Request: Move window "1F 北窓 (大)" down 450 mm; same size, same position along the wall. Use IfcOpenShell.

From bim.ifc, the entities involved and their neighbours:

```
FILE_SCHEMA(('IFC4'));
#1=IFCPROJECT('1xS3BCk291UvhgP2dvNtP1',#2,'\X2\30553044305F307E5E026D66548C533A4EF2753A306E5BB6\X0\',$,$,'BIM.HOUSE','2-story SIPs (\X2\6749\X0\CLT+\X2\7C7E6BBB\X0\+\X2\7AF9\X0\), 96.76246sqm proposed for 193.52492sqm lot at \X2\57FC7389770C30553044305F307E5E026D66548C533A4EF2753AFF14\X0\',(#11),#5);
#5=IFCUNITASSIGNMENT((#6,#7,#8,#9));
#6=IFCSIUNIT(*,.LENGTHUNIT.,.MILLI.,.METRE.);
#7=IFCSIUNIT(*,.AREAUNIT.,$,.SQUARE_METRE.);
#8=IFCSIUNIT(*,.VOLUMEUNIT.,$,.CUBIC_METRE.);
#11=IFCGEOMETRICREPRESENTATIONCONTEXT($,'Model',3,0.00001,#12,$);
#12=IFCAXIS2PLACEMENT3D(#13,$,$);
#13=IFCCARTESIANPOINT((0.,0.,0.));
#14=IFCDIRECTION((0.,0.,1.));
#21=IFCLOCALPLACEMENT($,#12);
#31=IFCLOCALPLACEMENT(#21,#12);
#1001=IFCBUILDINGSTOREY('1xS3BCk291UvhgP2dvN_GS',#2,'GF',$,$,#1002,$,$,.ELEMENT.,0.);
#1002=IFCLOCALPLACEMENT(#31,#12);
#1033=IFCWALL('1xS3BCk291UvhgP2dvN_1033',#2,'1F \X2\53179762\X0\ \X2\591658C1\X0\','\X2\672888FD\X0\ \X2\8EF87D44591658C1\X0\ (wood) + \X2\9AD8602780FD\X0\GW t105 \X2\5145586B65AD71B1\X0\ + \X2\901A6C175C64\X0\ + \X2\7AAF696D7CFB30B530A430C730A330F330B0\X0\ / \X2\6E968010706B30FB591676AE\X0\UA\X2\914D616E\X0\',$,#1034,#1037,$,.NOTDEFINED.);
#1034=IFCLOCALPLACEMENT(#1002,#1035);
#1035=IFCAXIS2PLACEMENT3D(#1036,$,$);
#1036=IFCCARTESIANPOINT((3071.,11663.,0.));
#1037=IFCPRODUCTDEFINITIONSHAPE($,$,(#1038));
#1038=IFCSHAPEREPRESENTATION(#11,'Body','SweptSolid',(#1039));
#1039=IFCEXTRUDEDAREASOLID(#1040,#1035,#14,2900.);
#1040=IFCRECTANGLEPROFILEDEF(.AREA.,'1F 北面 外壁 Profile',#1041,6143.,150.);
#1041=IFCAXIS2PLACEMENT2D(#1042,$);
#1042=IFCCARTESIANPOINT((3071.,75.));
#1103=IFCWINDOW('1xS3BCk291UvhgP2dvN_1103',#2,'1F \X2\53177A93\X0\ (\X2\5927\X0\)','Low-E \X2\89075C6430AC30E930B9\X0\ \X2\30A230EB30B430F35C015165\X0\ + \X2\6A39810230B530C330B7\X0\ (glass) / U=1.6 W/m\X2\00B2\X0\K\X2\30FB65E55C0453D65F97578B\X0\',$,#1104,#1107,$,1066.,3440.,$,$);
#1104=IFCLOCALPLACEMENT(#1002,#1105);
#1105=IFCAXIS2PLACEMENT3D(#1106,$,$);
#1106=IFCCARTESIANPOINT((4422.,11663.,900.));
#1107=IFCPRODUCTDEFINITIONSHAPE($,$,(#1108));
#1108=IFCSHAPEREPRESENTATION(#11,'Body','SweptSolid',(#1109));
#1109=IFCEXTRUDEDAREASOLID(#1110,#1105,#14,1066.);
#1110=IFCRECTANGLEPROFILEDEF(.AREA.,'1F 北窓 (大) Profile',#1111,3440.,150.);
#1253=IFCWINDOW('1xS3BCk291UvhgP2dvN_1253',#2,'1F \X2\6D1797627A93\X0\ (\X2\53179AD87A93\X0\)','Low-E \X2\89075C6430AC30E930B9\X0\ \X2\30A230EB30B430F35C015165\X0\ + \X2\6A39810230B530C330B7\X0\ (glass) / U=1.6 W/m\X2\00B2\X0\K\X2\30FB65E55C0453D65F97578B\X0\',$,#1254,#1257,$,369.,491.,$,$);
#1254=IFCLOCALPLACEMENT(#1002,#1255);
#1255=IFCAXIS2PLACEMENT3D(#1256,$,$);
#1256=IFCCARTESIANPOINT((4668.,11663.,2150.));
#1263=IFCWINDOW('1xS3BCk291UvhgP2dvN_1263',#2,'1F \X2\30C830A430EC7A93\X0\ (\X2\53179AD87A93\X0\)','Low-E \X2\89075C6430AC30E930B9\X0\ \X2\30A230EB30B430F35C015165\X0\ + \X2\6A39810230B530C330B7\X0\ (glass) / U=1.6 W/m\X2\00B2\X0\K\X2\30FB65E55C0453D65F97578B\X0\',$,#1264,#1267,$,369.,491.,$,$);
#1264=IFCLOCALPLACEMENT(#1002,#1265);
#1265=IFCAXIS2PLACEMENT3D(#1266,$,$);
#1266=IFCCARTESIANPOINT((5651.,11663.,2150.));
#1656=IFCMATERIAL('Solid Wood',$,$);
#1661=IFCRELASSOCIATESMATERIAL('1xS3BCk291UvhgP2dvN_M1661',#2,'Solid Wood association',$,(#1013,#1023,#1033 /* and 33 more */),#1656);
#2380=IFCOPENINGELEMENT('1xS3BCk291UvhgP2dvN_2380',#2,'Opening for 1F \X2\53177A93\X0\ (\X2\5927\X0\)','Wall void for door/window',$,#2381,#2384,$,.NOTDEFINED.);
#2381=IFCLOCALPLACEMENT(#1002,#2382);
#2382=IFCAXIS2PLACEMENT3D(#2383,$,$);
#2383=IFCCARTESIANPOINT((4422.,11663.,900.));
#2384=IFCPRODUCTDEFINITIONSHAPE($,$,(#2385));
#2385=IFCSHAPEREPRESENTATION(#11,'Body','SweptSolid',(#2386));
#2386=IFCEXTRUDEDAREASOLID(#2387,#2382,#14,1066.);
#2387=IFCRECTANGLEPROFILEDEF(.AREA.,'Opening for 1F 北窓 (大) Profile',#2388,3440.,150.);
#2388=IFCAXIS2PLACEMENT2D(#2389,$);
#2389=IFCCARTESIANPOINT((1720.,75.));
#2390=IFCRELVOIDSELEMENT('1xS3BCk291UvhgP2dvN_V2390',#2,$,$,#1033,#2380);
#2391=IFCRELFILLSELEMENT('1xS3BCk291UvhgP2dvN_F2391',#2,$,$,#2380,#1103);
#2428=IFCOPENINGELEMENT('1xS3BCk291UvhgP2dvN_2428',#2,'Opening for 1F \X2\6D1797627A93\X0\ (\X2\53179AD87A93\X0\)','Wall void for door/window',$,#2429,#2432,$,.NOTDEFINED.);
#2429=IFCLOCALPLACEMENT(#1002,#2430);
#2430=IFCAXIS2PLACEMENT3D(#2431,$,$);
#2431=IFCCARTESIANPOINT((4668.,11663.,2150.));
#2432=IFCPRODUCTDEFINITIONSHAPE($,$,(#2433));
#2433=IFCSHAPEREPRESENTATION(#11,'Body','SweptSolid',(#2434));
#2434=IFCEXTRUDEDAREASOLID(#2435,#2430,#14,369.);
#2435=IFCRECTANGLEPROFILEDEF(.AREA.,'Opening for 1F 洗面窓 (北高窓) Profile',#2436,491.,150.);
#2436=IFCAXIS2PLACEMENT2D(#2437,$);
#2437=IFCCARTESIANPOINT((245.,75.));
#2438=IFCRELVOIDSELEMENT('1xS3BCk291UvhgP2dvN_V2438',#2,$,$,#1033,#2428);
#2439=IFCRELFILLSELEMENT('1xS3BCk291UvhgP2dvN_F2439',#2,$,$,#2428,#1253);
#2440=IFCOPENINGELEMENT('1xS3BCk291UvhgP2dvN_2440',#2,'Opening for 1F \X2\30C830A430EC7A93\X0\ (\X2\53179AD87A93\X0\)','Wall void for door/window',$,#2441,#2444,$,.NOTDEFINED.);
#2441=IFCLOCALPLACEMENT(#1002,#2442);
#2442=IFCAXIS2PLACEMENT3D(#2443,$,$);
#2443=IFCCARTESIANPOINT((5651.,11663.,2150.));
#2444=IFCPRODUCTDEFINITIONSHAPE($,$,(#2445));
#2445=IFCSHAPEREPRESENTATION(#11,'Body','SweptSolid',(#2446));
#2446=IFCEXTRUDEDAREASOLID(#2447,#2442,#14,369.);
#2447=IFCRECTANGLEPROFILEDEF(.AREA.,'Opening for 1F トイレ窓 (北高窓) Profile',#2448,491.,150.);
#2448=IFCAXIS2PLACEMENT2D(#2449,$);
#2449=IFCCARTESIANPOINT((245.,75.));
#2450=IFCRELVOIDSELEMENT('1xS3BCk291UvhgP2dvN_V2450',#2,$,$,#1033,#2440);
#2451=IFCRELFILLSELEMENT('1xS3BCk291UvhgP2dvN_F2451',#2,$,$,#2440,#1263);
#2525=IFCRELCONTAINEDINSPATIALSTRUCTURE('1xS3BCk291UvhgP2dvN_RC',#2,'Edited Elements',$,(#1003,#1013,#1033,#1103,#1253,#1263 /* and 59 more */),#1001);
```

```python
import numpy as np
import ifcopenshell
import ifcopenshell.api.geometry
import ifcopenshell.util.placement
import ifcopenshell.util.unit

model = ifcopenshell.open("bim.ifc")
unit_scale = ifcopenshell.util.unit.calculate_unit_scale(model)

window = model.by_guid("1xS3BCk291UvhgP2dvN_1103")
opening = window.FillsVoids[0].RelatingOpeningElement
dz = -0.45 / unit_scale

shift = np.array([0.0, 0.0, dz])
# The window is not placed relative to its opening, so move both.
for product in (opening, window):
    matrix = ifcopenshell.util.placement.get_local_placement(product.ObjectPlacement)
    matrix[:3, 3] += shift
    ifcopenshell.api.geometry.edit_object_placement(model, product=product, matrix=matrix, is_si=False)

print(f"moved by {dz * unit_scale:+.3f} m")

model.write("bim_updated.ifc")
```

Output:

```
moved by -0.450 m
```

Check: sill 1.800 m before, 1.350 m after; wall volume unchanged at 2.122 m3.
